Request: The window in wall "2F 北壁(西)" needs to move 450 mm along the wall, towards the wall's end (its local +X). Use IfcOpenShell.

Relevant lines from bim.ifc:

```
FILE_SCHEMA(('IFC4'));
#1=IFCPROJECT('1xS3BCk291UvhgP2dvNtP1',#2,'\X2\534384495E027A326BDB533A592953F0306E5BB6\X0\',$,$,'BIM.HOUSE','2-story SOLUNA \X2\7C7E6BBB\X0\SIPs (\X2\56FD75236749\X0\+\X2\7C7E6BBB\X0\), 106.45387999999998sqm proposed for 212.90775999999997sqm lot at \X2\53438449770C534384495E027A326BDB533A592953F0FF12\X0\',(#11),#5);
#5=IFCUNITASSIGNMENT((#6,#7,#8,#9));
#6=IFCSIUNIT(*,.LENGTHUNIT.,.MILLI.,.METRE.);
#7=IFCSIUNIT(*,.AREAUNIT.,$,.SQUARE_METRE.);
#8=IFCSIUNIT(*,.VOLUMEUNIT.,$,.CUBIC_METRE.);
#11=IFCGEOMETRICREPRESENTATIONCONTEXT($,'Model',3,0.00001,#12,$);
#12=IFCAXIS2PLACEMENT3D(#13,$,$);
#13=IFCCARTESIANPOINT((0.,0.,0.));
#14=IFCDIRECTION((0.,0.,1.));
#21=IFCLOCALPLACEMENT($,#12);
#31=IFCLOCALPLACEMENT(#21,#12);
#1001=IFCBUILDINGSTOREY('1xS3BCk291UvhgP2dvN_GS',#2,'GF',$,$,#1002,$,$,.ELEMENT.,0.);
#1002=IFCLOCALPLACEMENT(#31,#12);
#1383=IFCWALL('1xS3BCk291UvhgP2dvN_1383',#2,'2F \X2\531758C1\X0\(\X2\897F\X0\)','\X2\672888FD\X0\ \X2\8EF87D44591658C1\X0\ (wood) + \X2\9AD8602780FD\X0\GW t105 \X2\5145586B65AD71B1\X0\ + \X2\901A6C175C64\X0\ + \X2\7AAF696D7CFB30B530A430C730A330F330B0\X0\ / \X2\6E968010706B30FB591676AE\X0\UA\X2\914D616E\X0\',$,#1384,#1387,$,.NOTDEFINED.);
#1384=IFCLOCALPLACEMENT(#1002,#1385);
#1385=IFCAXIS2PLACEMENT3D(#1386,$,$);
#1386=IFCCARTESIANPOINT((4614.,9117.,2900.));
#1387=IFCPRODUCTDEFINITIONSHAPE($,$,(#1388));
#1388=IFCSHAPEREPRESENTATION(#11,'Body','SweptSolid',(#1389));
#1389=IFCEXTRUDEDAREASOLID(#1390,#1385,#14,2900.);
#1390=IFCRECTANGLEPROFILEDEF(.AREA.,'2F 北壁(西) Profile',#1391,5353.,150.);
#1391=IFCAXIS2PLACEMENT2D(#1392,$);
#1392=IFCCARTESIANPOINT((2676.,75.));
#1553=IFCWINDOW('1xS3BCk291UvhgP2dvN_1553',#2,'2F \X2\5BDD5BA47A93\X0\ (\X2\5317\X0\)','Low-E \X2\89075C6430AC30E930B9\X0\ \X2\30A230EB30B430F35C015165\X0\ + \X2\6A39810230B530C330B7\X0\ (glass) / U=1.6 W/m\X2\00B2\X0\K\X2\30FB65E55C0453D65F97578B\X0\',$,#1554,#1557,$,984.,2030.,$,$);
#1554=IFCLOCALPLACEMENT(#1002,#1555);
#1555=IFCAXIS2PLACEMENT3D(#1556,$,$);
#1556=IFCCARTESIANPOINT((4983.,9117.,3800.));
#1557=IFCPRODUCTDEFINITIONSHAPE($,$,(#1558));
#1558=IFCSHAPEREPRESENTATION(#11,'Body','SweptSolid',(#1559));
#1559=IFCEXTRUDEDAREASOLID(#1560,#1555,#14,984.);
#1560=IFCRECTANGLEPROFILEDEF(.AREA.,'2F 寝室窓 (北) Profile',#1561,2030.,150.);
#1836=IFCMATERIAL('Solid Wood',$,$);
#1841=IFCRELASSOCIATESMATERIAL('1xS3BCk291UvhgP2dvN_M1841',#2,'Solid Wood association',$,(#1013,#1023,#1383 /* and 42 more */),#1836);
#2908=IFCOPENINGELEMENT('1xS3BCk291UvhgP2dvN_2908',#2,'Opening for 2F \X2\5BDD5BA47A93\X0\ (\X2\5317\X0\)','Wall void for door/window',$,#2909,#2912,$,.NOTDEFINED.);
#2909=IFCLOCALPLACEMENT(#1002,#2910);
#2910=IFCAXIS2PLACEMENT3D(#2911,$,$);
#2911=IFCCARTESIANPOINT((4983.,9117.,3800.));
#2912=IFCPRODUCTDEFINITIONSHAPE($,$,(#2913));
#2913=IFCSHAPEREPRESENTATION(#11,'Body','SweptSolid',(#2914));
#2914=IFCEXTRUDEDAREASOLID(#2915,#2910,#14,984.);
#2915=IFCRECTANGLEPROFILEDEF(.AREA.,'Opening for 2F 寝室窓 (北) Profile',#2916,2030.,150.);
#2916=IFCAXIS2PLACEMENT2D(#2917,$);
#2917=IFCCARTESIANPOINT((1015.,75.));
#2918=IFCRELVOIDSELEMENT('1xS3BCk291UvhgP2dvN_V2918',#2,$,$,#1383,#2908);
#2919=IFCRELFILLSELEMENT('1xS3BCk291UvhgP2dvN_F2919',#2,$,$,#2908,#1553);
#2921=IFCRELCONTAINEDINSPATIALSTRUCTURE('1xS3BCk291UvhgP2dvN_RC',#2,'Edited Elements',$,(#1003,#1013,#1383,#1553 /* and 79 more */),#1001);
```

```python
import ifcopenshell
import ifcopenshell.api.geometry
import ifcopenshell.util.placement
import ifcopenshell.util.unit

model = ifcopenshell.open("bim.ifc")
unit_scale = ifcopenshell.util.unit.calculate_unit_scale(model)

window = model.by_guid("1xS3BCk291UvhgP2dvN_1553")
opening = window.FillsVoids[0].RelatingOpeningElement
wall = opening.VoidsElements[0].RelatingBuildingElement

wall_matrix = ifcopenshell.util.placement.get_local_placement(wall.ObjectPlacement)
shift = wall_matrix[:3, 0] * 0.45 / unit_scale
before = ifcopenshell.util.placement.get_local_placement(window.ObjectPlacement)[:3, 3].copy()

# The window is not placed relative to its opening, so move both.
for product in (opening, window):
    matrix = ifcopenshell.util.placement.get_local_placement(product.ObjectPlacement)
    matrix[:3, 3] += shift
    ifcopenshell.api.geometry.edit_object_placement(model, product=product, matrix=matrix, is_si=False)

after = ifcopenshell.util.placement.get_local_placement(window.ObjectPlacement)[:3, 3]
print("window moved by", (after - before).round(3) + 0.0)

model.write("bim_v2.ifc")
```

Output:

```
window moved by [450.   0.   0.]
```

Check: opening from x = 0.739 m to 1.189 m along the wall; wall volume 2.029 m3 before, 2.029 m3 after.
